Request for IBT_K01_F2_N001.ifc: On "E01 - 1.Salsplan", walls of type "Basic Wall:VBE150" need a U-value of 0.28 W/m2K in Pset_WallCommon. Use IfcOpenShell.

First a look at what the model holds.

```python
import ifcopenshell
import ifcopenshell.util.element

model = ifcopenshell.open("IBT_K01_F2_N001.ifc")
print(model.schema)
storey = next(s for s in model.by_type("IfcBuildingStorey") if s.Name == "E01 - 1.Salsplan")
walls = [e for e in ifcopenshell.util.element.get_decomposition(storey) if e.is_a("IfcWall")]
seen = {}
for e in walls:
    element_type = ifcopenshell.util.element.get_type(e)
    key = (element_type.Name if element_type != e and element_type else None, ifcopenshell.util.element.get_pset(e, "Pset_WallCommon", "ThermalTransmittance"))
    seen[key] = seen.get(key, 0) + 1
for (name, value), count in sorted(seen.items(), key=str):
    print(count, "x", name, "|", value)
```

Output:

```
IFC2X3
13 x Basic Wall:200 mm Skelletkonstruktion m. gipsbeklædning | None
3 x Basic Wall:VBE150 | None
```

```python
import ifcopenshell
import ifcopenshell.api.pset
import ifcopenshell.util.element

model = ifcopenshell.open("IBT_K01_F2_N001.ifc")

storey = next(s for s in model.by_type("IfcBuildingStorey") if s.Name == "E01 - 1.Salsplan")
walls = [e for e in ifcopenshell.util.element.get_decomposition(storey) if e.is_a("IfcWall")]

count = 0
for e in walls:
    element_type = ifcopenshell.util.element.get_type(e)
    if element_type in (None, e) or element_type.Name != "Basic Wall:VBE150":
        continue
    # add_pset returns the element's existing set when there is one.
    pset = ifcopenshell.api.pset.add_pset(model, product=e, name="Pset_WallCommon")
    ifcopenshell.api.pset.edit_pset(model, pset=pset, properties={"ThermalTransmittance": 0.28})
    count += 1

print(count, "walls updated")

model.write("IBT_K01_F2_N001_updated.ifc")
```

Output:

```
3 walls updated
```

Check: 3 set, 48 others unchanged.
